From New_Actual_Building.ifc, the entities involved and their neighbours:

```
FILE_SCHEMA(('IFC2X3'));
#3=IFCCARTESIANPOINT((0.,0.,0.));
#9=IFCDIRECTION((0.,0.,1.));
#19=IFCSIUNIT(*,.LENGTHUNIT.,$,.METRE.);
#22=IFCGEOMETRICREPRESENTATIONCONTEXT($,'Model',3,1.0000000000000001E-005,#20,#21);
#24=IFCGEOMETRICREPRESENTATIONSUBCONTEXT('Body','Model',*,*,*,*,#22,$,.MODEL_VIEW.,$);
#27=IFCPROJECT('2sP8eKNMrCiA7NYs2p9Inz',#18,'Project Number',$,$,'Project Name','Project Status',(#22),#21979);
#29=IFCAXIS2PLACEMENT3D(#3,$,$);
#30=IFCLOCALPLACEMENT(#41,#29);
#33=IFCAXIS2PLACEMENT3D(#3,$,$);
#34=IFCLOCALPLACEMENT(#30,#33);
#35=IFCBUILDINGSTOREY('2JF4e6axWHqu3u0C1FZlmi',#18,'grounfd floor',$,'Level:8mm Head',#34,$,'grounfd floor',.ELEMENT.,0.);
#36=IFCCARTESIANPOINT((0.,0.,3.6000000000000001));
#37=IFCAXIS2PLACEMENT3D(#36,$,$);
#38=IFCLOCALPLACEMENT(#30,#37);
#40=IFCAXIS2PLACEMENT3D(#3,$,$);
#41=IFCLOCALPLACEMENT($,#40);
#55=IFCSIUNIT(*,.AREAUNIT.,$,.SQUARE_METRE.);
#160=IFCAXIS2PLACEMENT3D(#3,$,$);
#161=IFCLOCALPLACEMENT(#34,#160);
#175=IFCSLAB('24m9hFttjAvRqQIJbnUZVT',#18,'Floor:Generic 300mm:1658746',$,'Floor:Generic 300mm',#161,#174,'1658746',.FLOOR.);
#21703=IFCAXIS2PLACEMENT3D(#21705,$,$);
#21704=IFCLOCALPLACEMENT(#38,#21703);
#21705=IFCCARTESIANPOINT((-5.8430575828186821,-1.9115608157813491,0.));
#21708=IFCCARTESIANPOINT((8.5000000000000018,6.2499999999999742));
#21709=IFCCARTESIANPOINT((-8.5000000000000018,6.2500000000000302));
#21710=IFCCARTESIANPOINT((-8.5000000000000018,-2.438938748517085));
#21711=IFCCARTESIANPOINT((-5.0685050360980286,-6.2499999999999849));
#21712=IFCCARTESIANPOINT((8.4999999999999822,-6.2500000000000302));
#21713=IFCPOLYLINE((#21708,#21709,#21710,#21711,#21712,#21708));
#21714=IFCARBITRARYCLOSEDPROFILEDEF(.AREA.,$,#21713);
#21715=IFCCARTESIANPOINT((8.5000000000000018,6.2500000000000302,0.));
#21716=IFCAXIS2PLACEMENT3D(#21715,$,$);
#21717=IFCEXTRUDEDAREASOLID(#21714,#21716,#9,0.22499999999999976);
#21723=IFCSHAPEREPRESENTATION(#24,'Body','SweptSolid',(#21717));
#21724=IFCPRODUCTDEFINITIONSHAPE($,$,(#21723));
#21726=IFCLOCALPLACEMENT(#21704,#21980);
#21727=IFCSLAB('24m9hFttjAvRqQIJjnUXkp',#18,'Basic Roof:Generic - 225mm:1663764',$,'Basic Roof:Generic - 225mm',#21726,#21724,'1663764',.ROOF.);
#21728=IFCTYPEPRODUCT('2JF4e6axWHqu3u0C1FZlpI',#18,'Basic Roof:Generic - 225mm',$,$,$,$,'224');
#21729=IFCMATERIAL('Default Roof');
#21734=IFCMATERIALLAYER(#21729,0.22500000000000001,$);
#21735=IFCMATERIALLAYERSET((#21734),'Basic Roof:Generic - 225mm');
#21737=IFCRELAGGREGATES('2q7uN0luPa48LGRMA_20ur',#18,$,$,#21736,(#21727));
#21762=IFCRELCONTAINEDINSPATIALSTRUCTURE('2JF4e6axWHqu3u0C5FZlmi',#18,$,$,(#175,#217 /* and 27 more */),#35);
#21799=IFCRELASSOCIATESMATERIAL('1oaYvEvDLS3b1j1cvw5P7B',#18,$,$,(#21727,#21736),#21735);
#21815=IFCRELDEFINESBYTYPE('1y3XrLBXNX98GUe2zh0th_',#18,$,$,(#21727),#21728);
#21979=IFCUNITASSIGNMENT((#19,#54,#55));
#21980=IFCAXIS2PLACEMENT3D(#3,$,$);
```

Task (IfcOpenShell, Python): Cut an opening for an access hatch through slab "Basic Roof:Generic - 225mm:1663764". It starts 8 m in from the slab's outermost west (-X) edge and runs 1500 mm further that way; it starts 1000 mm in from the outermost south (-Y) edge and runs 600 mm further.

```python
import numpy as np
import ifcopenshell
import ifcopenshell.api.feature
import ifcopenshell.api.geometry
import ifcopenshell.api.root
import ifcopenshell.geom
import ifcopenshell.util.placement
import ifcopenshell.util.representation
import ifcopenshell.util.shape
import ifcopenshell.util.unit

model = ifcopenshell.open("New_Actual_Building.ifc")
unit_scale = ifcopenshell.util.unit.calculate_unit_scale(model)
settings = ifcopenshell.geom.settings()


def volume(element):
    """Net volume in cubic metres, openings subtracted."""
    shape = ifcopenshell.geom.create_shape(settings, element)
    return ifcopenshell.util.shape.get_volume(shape.geometry)


slab = model.by_guid("24m9hFttjAvRqQIJjnUXkp")
before = volume(slab)

# Extent in the slab's own axes, in metres. The edges named are its -X and -Y sides.
slab_shape = ifcopenshell.geom.create_shape(settings, slab)
vertices = ifcopenshell.util.shape.get_vertices(slab_shape.geometry)
x_min, y_min, bottom = vertices.min(axis=0)
top = vertices[:, 2].max()

opening = ifcopenshell.api.root.create_entity(model, ifc_class="IfcOpeningElement", name="Access hatch opening")
context = ifcopenshell.util.representation.get_context(model, "Model", "Body", "MODEL_VIEW")
width, depth = 1.5, 0.6
outline = [(0.0, 0.0), (width, 0.0), (width, depth), (0.0, depth), (0.0, 0.0)]
# Overshoot both faces by 50 mm so the cut is clean.
shape = ifcopenshell.api.geometry.add_slab_representation(
    model, context=context, depth=top - bottom + 0.1, polyline=outline
)
ifcopenshell.api.geometry.assign_representation(model, product=opening, representation=shape)

matrix = ifcopenshell.util.placement.get_local_placement(slab.ObjectPlacement)
matrix[:, 3] = matrix @ np.append(np.array([x_min + 8, y_min + 1, bottom - 0.05]) / unit_scale, 1.0)
ifcopenshell.api.geometry.edit_object_placement(model, product=opening, matrix=matrix, is_si=False)
ifcopenshell.api.feature.add_feature(model, feature=opening, element=slab)

after = volume(slab)

print(f"slab volume {before:.3f} -> {after:.3f} m3")

model.write("New_Actual_Building_rev.ifc")
```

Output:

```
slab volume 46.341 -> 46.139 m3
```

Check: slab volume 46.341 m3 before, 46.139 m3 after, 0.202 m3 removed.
